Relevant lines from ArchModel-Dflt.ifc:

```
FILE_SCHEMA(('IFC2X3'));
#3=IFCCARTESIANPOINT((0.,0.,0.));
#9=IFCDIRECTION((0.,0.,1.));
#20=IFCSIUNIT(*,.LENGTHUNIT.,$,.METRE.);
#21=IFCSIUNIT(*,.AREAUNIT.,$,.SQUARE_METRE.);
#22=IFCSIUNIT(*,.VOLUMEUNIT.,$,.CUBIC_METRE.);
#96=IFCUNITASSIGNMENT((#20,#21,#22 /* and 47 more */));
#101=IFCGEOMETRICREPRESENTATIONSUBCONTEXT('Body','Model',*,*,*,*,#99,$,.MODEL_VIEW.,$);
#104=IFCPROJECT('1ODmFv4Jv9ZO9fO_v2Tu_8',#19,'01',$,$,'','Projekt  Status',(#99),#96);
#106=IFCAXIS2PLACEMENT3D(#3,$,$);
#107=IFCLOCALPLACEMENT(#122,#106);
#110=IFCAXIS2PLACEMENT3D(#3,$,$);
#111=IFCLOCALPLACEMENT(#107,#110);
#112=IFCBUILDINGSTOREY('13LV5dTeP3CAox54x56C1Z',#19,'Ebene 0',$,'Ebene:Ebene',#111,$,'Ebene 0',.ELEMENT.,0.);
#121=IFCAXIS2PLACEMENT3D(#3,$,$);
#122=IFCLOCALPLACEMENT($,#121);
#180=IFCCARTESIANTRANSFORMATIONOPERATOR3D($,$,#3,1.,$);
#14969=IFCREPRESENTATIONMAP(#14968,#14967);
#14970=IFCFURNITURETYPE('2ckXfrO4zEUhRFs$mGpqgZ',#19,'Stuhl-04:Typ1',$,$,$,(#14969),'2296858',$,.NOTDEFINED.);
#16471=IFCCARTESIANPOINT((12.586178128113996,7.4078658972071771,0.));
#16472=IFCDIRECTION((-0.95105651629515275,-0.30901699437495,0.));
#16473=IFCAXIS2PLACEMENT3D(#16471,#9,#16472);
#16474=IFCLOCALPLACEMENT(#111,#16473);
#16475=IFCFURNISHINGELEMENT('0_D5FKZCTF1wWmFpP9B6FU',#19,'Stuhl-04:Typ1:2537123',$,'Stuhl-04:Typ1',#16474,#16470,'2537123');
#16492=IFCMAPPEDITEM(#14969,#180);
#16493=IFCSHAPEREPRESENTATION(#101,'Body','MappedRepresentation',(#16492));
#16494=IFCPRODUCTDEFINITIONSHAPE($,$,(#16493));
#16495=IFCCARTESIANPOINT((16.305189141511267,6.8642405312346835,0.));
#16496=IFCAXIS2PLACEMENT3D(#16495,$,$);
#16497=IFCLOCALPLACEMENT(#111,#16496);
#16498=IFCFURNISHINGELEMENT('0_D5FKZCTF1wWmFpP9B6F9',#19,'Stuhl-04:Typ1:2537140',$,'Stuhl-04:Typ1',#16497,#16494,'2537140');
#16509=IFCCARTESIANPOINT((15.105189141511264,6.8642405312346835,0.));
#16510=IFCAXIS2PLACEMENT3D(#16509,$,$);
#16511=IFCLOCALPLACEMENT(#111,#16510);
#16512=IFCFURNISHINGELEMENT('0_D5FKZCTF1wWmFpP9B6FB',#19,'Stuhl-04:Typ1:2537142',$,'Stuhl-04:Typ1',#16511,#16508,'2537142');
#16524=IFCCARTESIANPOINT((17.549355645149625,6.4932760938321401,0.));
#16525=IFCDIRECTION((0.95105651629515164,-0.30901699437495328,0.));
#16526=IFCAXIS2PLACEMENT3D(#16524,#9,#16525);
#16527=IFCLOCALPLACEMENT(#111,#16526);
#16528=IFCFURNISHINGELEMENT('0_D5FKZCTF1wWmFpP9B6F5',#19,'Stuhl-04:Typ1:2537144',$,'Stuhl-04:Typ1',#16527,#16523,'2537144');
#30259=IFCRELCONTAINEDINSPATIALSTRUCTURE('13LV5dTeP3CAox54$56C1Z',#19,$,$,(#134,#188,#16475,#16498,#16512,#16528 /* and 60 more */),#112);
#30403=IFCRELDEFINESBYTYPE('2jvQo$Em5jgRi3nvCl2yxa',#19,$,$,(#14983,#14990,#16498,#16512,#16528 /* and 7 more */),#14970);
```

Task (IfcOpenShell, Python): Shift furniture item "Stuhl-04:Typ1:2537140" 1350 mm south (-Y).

```python
import ifcopenshell
import ifcopenshell.api.geometry
import ifcopenshell.util.placement
import ifcopenshell.util.unit

model = ifcopenshell.open("ArchModel-Dflt.ifc")
unit_scale = ifcopenshell.util.unit.calculate_unit_scale(model)

item = model.by_guid("0_D5FKZCTF1wWmFpP9B6F9")
matrix = ifcopenshell.util.placement.get_local_placement(item.ObjectPlacement)
matrix[1, 3] -= 1.35 / unit_scale
ifcopenshell.api.geometry.edit_object_placement(model, product=item, matrix=matrix, is_si=False)

print(ifcopenshell.util.placement.get_local_placement(item.ObjectPlacement).round(3) + 0.0)

model.write("ArchModel-Dflt_edited.ifc")
```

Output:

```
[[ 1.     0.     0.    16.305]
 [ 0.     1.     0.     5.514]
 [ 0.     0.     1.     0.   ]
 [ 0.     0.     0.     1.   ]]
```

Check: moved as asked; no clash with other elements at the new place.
